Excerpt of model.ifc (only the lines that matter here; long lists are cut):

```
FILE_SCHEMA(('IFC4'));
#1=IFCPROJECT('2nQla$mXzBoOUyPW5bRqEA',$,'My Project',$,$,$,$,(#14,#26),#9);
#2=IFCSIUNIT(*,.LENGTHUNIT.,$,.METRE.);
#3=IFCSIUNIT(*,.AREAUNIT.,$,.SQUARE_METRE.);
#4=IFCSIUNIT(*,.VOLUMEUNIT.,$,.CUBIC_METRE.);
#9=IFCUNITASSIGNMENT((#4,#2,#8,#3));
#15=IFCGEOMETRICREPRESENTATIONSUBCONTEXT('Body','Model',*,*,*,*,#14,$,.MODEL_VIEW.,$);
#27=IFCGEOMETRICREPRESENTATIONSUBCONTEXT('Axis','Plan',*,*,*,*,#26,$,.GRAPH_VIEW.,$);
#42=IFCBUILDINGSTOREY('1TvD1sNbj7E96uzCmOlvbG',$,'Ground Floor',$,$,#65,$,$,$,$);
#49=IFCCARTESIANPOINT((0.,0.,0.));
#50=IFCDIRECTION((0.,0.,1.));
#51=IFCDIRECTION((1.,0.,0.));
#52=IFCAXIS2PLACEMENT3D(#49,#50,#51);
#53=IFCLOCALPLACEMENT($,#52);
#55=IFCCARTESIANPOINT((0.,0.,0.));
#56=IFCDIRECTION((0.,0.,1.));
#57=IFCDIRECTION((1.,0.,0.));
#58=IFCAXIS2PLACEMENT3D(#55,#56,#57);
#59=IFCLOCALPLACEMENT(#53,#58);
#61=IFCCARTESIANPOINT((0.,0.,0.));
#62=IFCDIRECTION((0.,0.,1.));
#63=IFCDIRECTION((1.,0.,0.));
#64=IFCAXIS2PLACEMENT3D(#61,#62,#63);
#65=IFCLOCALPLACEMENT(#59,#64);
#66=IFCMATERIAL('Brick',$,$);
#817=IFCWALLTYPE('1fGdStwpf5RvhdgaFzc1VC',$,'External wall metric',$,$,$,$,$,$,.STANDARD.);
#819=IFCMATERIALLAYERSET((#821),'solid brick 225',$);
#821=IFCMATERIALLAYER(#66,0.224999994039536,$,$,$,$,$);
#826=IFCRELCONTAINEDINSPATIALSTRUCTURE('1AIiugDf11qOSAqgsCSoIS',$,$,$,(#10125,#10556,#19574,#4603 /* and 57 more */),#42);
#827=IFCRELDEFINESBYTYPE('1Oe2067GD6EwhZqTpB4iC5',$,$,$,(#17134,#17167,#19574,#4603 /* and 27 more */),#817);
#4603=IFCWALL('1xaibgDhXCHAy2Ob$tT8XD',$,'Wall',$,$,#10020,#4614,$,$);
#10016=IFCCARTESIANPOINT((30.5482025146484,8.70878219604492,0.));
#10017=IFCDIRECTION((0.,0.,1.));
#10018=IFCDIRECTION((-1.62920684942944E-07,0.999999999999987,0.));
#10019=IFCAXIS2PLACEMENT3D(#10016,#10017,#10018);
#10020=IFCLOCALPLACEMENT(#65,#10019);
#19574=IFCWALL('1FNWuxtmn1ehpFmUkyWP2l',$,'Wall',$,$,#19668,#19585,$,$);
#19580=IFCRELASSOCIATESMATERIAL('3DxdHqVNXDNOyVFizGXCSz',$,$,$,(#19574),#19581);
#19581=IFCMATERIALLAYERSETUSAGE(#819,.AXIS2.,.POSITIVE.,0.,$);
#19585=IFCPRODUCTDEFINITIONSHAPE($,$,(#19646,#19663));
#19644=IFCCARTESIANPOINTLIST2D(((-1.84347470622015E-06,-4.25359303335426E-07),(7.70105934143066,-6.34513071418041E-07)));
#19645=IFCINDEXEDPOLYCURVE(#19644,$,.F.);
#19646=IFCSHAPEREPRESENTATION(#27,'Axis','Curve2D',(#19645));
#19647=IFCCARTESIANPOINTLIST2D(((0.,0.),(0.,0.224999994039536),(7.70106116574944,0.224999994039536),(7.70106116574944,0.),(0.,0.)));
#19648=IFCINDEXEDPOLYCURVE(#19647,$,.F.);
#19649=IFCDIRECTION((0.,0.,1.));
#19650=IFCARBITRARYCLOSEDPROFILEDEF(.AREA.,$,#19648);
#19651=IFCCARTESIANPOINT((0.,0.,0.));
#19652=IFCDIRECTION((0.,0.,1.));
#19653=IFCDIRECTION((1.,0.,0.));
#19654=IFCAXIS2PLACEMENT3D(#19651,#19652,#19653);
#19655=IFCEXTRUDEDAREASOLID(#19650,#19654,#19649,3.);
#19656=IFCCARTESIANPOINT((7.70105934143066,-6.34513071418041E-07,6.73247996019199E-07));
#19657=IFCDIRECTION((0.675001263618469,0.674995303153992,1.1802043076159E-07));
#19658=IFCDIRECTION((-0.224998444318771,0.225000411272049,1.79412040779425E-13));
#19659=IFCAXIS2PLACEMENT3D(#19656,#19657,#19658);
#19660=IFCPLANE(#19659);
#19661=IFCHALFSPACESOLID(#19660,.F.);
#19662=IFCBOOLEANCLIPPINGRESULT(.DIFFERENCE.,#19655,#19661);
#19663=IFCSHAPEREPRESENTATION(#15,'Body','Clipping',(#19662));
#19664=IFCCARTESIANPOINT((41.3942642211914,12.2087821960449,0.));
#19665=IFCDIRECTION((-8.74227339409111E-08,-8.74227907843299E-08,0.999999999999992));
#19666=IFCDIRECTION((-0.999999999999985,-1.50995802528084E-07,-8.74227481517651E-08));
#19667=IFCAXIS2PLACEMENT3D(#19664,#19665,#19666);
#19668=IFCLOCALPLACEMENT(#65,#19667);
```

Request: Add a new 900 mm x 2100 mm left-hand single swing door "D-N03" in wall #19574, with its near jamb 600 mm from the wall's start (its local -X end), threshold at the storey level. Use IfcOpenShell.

```python
import numpy as np
import ifcopenshell
import ifcopenshell.api.feature
import ifcopenshell.api.geometry
import ifcopenshell.api.root
import ifcopenshell.api.spatial
import ifcopenshell.geom
import ifcopenshell.util.element
import ifcopenshell.util.placement
import ifcopenshell.util.representation
import ifcopenshell.util.shape
import ifcopenshell.util.unit

model = ifcopenshell.open("model.ifc")
unit_scale = ifcopenshell.util.unit.calculate_unit_scale(model)
settings = ifcopenshell.geom.settings()


def volume(element):
    """Net volume in cubic metres, openings subtracted."""
    shape = ifcopenshell.geom.create_shape(settings, element)
    return ifcopenshell.util.shape.get_volume(shape.geometry)


wall = model.by_guid("1FNWuxtmn1ehpFmUkyWP2l")
storey = ifcopenshell.util.element.get_container(wall, ifc_class="IfcBuildingStorey")
context = ifcopenshell.util.representation.get_context(model, "Model", "Body", "MODEL_VIEW")
before = volume(wall)

width, height, from_end, sill = 0.9, 2.1, 0.6, 0.0  # metres

# The wall runs along its own X axis, and the end named is its -X end.
wall_shape = ifcopenshell.geom.create_shape(settings, wall)
x, y, z = ifcopenshell.util.shape.get_vertices(wall_shape.geometry).T
start = x.min() + from_end
face, thickness = float(y.min()), float(y.max() - y.min())
wall_matrix = ifcopenshell.util.placement.get_local_placement(wall.ObjectPlacement)
level = ifcopenshell.util.placement.get_local_placement(storey.ObjectPlacement)[2, 3]


def in_wall(x, y):
    """Placement at x, y metres in the wall's axes, at sill height."""
    matrix = wall_matrix.copy()
    matrix[:, 3] = wall_matrix @ np.array([x / unit_scale, y / unit_scale, 0.0, 1.0])
    matrix[2, 3] = level + sill / unit_scale
    return matrix


# Opening: a box that overshoots both wall faces by 50 mm.
opening = ifcopenshell.api.root.create_entity(model, ifc_class="IfcOpeningElement", predefined_type="OPENING")
box = ifcopenshell.api.geometry.add_wall_representation(
    model, context=context, length=width, height=height, thickness=thickness + 0.1
)
ifcopenshell.api.geometry.assign_representation(model, product=opening, representation=box)
ifcopenshell.api.geometry.edit_object_placement(model, product=opening, matrix=in_wall(start, face - 0.05), is_si=False)
ifcopenshell.api.feature.add_feature(model, feature=opening, element=wall)

door = ifcopenshell.api.root.create_entity(model, ifc_class="IfcDoor", name="D-N03", predefined_type="DOOR")
door.OverallWidth, door.OverallHeight = width / unit_scale, height / unit_scale
door.OperationType = "SINGLE_SWING_LEFT"
body = ifcopenshell.api.geometry.add_door_representation(
    model,
    context=context,
    overall_width=door.OverallWidth,
    overall_height=door.OverallHeight,
    operation_type="SINGLE_SWING_LEFT",
    lining_properties={"LiningDepth": thickness / unit_scale, "ThresholdDepth": thickness / unit_scale},
)
ifcopenshell.api.geometry.assign_representation(model, product=door, representation=body)
ifcopenshell.api.spatial.assign_container(model, products=[door], relating_structure=storey)
ifcopenshell.api.feature.add_filling(model, opening=opening, element=door)

# The lining spans the wall, so the door starts at the wall face.
ifcopenshell.api.geometry.edit_object_placement(model, product=door, matrix=in_wall(start, face), is_si=False)

after = volume(wall)

print(f"wall volume {before:.3f} -> {after:.3f} m3")

model.write("model_rev.ifc")
```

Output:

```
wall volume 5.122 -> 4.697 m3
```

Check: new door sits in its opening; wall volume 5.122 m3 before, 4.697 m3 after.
